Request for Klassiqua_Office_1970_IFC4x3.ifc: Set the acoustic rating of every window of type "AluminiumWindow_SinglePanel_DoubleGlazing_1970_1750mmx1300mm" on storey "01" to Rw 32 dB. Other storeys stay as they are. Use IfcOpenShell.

First a look at what the model holds.

```python
import ifcopenshell
import ifcopenshell.util.element

model = ifcopenshell.open("Klassiqua_Office_1970_IFC4x3.ifc")
print(model.schema)
storey = next(s for s in model.by_type("IfcBuildingStorey") if s.Name == "01")
windows = [e for e in ifcopenshell.util.element.get_decomposition(storey) if e.is_a("IfcWindow")]
seen = {}
for e in windows:
    element_type = ifcopenshell.util.element.get_type(e)
    key = (element_type.Name if element_type != e and element_type else None, ifcopenshell.util.element.get_pset(e, "Pset_WindowCommon", "AcousticRating"))
    seen[key] = seen.get(key, 0) + 1
for (name, value), count in sorted(seen.items(), key=str):
    print(count, "x", name, "|", value)
```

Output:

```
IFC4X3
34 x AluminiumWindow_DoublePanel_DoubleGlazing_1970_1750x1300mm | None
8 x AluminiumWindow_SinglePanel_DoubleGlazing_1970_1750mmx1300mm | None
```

```python
import ifcopenshell
import ifcopenshell.api.pset
import ifcopenshell.util.element

model = ifcopenshell.open("Klassiqua_Office_1970_IFC4x3.ifc")

storey = next(s for s in model.by_type("IfcBuildingStorey") if s.Name == "01")
windows = [e for e in ifcopenshell.util.element.get_decomposition(storey) if e.is_a("IfcWindow")]

count = 0
for e in windows:
    element_type = ifcopenshell.util.element.get_type(e)
    if element_type in (None, e) or element_type.Name != "AluminiumWindow_SinglePanel_DoubleGlazing_1970_1750mmx1300mm":
        continue
    # add_pset returns the element's existing set when there is one.
    pset = ifcopenshell.api.pset.add_pset(model, product=e, name="Pset_WindowCommon")
    ifcopenshell.api.pset.edit_pset(model, pset=pset, properties={"AcousticRating": "Rw 32 dB"})
    count += 1

print(count, "windows updated")

model.write("Klassiqua_Office_1970_IFC4x3_edited.ifc")
```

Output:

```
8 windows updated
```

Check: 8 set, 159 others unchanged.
